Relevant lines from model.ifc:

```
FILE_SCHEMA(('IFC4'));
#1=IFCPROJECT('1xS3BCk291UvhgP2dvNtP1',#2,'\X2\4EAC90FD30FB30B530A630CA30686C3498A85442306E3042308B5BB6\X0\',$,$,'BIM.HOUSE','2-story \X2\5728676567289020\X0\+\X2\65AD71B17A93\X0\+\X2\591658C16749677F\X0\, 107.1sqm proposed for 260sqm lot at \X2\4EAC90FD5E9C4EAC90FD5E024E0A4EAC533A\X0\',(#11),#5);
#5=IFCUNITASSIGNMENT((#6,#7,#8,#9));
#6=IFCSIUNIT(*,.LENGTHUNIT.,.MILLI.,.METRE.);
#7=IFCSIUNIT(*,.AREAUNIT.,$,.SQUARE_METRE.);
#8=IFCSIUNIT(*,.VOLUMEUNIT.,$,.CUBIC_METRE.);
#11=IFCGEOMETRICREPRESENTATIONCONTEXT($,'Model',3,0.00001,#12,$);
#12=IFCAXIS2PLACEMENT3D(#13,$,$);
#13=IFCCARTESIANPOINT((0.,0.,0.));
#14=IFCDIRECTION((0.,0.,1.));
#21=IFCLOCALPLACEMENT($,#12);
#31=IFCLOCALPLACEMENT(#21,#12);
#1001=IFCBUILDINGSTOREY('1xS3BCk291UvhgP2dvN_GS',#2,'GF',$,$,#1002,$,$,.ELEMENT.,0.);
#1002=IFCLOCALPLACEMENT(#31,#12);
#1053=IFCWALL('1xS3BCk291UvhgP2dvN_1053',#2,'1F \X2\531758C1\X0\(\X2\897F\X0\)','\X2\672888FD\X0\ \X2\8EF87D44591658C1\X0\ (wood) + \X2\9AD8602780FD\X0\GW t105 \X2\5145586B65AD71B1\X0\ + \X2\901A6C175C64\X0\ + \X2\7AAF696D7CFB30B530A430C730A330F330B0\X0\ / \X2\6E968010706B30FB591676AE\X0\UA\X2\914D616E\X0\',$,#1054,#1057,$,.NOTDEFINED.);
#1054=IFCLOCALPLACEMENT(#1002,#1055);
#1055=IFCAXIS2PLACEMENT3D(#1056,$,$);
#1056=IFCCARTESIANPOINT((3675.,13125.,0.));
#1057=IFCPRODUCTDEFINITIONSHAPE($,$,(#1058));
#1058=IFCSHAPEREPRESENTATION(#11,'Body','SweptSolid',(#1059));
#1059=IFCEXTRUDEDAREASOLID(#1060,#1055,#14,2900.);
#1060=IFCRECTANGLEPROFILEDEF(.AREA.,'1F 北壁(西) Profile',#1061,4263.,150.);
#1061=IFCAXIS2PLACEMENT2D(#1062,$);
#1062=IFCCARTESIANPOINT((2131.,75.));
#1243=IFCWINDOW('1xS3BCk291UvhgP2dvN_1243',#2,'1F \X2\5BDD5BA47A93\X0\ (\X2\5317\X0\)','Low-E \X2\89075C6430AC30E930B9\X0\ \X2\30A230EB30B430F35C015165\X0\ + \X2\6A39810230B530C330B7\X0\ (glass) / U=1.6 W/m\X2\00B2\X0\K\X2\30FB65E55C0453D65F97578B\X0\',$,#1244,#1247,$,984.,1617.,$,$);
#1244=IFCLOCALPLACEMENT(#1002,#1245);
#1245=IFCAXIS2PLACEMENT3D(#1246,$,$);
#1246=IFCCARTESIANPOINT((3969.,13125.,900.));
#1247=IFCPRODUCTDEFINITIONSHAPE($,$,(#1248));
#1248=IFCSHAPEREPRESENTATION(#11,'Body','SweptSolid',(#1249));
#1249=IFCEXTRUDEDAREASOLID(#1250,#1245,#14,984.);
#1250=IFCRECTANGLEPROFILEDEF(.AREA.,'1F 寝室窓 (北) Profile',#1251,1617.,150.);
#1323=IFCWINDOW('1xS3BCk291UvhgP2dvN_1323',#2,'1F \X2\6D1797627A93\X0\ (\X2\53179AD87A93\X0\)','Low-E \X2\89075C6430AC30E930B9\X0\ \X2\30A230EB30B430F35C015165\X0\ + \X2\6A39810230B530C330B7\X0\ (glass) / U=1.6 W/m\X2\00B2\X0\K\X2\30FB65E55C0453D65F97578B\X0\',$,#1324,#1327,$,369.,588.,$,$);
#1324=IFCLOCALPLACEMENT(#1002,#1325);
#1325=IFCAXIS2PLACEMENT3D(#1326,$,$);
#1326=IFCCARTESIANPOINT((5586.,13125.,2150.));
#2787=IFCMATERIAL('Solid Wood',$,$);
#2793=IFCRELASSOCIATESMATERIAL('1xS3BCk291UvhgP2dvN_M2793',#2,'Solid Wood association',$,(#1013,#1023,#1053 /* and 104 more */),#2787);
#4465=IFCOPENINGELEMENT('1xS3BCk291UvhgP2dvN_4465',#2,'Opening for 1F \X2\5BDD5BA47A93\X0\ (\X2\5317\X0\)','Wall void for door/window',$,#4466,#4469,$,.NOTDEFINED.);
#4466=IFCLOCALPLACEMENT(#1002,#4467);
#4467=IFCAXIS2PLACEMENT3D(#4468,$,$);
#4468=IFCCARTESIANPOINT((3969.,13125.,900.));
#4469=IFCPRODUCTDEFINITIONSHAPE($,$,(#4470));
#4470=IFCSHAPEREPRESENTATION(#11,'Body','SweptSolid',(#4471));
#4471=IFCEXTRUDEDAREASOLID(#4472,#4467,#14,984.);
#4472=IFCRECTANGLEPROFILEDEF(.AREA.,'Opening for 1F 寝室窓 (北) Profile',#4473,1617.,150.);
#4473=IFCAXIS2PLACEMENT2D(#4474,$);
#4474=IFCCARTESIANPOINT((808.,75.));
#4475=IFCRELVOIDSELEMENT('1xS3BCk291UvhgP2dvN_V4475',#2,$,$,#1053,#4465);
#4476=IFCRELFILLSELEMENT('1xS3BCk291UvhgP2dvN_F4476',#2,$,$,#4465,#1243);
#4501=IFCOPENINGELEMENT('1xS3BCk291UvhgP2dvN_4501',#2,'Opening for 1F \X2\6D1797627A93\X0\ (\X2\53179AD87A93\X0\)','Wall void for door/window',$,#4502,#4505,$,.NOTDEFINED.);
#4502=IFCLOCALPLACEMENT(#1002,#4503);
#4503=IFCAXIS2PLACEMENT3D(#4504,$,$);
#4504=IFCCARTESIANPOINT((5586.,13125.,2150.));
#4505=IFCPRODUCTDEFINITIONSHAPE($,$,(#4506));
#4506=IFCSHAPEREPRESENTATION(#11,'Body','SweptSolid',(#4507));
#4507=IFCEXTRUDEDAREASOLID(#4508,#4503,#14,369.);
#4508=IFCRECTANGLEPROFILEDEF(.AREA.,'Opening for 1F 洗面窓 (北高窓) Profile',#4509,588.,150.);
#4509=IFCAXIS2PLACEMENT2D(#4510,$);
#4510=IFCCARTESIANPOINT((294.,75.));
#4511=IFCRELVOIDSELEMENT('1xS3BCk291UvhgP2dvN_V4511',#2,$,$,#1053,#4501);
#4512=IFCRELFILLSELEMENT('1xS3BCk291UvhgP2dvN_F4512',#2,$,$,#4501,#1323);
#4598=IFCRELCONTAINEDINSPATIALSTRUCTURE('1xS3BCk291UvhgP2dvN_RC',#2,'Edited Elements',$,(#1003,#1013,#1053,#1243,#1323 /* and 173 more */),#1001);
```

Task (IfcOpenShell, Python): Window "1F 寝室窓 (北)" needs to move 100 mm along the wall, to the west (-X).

```python
import ifcopenshell
import ifcopenshell.api.geometry
import ifcopenshell.util.placement

model = ifcopenshell.open("model.ifc")

window = model.by_guid("1xS3BCk291UvhgP2dvN_1243")
opening = window.FillsVoids[0].RelatingOpeningElement
wall = opening.VoidsElements[0].RelatingBuildingElement

wall_matrix = ifcopenshell.util.placement.get_local_placement(wall.ObjectPlacement)
shift = wall_matrix[:3, 0] * -100.0
before = ifcopenshell.util.placement.get_local_placement(window.ObjectPlacement)[:3, 3].copy()

# The window is not placed relative to its opening, so move both.
for product in (opening, window):
    matrix = ifcopenshell.util.placement.get_local_placement(product.ObjectPlacement)
    matrix[:3, 3] += shift
    ifcopenshell.api.geometry.edit_object_placement(model, product=product, matrix=matrix, is_si=False)

after = ifcopenshell.util.placement.get_local_placement(window.ObjectPlacement)[:3, 3]
print("window moved by", (after - before).round(3) + 0.0)

model.write("model_updated.ifc")
```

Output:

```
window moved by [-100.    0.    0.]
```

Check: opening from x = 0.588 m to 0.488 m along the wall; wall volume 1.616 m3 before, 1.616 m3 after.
